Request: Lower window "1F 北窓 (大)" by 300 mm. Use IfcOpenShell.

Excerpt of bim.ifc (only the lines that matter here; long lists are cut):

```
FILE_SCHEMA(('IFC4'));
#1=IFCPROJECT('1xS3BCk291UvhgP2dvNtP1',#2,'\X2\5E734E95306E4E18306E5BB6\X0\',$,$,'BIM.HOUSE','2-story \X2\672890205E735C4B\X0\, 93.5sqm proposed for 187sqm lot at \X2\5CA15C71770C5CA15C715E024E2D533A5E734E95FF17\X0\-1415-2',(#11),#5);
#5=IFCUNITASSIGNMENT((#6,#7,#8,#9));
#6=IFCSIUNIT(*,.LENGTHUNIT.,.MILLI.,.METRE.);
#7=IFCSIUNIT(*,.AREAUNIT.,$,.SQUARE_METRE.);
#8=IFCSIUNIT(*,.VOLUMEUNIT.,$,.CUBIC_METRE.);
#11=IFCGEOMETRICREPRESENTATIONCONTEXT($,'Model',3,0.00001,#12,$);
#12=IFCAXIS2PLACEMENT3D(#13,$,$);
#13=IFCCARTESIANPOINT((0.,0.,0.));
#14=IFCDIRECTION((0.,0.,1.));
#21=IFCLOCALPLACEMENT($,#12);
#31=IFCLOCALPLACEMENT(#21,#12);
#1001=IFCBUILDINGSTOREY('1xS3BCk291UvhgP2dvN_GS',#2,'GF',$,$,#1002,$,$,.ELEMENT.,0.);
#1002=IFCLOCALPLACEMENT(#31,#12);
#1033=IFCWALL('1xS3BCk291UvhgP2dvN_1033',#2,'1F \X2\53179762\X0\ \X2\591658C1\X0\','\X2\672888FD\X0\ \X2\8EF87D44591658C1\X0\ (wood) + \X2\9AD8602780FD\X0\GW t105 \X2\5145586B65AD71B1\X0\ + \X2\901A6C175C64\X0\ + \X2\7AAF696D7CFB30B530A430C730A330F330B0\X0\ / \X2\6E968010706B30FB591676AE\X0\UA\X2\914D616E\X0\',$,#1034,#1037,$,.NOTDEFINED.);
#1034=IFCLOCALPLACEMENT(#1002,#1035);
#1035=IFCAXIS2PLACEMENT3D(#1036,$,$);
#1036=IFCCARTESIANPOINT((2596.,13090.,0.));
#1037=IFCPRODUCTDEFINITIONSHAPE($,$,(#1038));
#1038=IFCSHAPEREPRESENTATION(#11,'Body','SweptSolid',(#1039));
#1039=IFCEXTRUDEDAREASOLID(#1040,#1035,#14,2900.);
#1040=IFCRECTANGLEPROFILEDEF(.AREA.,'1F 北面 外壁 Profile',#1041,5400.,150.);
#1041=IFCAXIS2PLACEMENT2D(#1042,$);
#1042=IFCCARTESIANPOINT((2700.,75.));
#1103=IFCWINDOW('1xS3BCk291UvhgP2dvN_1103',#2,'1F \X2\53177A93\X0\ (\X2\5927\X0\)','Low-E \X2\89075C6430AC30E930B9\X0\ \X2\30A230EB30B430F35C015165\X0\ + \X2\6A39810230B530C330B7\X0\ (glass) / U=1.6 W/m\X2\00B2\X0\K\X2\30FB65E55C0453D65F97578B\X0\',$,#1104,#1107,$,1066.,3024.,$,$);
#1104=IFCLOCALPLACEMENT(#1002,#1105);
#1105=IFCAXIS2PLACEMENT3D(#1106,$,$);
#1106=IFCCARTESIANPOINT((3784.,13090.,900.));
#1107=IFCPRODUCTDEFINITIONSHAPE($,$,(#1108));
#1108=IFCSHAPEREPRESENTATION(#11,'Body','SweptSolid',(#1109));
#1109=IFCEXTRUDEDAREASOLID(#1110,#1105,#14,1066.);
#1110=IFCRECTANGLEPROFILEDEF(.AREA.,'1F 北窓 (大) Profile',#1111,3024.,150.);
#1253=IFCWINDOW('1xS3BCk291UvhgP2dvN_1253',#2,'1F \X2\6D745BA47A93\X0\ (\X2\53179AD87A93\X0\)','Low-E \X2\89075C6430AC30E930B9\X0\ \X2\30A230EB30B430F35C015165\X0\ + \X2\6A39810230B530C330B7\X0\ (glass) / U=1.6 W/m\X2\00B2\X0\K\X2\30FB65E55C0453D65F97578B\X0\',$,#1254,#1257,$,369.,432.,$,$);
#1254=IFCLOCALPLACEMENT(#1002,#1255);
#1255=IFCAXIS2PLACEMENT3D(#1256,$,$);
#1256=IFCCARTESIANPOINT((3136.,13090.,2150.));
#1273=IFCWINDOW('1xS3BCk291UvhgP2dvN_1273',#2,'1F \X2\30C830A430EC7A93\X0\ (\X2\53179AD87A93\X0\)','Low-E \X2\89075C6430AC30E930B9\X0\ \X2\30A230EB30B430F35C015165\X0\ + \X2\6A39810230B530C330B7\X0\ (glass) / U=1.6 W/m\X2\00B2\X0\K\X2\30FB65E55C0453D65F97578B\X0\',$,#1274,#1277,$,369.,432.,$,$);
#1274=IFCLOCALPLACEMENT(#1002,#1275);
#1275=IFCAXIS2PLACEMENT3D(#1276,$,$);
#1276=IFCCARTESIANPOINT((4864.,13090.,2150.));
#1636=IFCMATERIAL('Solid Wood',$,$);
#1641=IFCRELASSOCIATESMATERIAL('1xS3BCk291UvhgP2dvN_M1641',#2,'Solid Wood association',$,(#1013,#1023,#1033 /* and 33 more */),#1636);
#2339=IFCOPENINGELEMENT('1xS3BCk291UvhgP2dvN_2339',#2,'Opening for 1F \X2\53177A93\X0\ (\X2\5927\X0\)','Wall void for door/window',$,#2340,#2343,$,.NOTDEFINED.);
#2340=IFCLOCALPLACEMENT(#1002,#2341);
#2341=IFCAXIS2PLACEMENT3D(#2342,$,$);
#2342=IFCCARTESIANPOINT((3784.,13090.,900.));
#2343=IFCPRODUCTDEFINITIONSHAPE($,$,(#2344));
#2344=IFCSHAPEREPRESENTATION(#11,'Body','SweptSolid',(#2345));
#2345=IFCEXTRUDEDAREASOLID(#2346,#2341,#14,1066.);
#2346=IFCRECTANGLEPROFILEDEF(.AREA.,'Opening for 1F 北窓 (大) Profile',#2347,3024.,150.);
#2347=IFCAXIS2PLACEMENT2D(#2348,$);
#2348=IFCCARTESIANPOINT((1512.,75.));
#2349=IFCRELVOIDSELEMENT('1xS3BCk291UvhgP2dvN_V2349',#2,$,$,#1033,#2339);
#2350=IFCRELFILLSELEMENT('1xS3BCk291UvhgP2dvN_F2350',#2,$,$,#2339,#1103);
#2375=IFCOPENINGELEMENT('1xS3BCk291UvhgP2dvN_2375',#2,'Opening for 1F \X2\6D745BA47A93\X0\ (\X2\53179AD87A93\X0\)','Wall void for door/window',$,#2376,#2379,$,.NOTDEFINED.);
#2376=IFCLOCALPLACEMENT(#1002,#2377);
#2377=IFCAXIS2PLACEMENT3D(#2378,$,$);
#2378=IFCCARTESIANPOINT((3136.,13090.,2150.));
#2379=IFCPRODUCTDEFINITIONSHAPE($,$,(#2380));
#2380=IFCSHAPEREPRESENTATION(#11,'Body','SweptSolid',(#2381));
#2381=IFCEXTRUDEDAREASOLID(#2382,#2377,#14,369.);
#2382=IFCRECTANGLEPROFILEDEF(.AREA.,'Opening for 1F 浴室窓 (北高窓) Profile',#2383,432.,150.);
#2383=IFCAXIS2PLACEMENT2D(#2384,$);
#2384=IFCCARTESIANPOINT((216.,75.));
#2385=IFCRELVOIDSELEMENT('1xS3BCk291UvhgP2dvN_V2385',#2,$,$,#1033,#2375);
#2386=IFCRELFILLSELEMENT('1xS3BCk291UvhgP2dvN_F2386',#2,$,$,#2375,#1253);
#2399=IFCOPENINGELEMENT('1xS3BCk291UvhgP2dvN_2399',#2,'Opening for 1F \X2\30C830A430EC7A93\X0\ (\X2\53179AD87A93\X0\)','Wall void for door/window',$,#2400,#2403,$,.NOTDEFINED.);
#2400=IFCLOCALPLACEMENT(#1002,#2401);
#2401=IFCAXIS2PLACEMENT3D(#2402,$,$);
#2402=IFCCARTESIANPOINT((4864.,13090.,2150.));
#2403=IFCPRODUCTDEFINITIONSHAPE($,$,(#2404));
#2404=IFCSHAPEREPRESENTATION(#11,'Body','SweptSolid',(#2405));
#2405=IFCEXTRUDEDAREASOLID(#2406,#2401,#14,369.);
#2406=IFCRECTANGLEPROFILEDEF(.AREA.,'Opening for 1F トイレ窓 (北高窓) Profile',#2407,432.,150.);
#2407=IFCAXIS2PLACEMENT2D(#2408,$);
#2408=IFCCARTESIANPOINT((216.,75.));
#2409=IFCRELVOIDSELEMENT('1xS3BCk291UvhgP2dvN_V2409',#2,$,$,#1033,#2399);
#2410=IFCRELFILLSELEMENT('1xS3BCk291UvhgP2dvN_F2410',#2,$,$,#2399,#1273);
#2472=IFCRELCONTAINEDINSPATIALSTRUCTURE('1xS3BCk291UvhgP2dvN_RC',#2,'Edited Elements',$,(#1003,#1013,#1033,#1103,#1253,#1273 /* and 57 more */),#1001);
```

```python
import numpy as np
import ifcopenshell
import ifcopenshell.api.geometry
import ifcopenshell.util.placement
import ifcopenshell.util.unit

model = ifcopenshell.open("bim.ifc")
unit_scale = ifcopenshell.util.unit.calculate_unit_scale(model)

window = model.by_guid("1xS3BCk291UvhgP2dvN_1103")
opening = window.FillsVoids[0].RelatingOpeningElement
dz = -0.3 / unit_scale

shift = np.array([0.0, 0.0, dz])
# The window is not placed relative to its opening, so move both.
for product in (opening, window):
    matrix = ifcopenshell.util.placement.get_local_placement(product.ObjectPlacement)
    matrix[:3, 3] += shift
    ifcopenshell.api.geometry.edit_object_placement(model, product=product, matrix=matrix, is_si=False)

print(f"moved by {dz * unit_scale:+.3f} m")

model.write("bim_updated.ifc")
```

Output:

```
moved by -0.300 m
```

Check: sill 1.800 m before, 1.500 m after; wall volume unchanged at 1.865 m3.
